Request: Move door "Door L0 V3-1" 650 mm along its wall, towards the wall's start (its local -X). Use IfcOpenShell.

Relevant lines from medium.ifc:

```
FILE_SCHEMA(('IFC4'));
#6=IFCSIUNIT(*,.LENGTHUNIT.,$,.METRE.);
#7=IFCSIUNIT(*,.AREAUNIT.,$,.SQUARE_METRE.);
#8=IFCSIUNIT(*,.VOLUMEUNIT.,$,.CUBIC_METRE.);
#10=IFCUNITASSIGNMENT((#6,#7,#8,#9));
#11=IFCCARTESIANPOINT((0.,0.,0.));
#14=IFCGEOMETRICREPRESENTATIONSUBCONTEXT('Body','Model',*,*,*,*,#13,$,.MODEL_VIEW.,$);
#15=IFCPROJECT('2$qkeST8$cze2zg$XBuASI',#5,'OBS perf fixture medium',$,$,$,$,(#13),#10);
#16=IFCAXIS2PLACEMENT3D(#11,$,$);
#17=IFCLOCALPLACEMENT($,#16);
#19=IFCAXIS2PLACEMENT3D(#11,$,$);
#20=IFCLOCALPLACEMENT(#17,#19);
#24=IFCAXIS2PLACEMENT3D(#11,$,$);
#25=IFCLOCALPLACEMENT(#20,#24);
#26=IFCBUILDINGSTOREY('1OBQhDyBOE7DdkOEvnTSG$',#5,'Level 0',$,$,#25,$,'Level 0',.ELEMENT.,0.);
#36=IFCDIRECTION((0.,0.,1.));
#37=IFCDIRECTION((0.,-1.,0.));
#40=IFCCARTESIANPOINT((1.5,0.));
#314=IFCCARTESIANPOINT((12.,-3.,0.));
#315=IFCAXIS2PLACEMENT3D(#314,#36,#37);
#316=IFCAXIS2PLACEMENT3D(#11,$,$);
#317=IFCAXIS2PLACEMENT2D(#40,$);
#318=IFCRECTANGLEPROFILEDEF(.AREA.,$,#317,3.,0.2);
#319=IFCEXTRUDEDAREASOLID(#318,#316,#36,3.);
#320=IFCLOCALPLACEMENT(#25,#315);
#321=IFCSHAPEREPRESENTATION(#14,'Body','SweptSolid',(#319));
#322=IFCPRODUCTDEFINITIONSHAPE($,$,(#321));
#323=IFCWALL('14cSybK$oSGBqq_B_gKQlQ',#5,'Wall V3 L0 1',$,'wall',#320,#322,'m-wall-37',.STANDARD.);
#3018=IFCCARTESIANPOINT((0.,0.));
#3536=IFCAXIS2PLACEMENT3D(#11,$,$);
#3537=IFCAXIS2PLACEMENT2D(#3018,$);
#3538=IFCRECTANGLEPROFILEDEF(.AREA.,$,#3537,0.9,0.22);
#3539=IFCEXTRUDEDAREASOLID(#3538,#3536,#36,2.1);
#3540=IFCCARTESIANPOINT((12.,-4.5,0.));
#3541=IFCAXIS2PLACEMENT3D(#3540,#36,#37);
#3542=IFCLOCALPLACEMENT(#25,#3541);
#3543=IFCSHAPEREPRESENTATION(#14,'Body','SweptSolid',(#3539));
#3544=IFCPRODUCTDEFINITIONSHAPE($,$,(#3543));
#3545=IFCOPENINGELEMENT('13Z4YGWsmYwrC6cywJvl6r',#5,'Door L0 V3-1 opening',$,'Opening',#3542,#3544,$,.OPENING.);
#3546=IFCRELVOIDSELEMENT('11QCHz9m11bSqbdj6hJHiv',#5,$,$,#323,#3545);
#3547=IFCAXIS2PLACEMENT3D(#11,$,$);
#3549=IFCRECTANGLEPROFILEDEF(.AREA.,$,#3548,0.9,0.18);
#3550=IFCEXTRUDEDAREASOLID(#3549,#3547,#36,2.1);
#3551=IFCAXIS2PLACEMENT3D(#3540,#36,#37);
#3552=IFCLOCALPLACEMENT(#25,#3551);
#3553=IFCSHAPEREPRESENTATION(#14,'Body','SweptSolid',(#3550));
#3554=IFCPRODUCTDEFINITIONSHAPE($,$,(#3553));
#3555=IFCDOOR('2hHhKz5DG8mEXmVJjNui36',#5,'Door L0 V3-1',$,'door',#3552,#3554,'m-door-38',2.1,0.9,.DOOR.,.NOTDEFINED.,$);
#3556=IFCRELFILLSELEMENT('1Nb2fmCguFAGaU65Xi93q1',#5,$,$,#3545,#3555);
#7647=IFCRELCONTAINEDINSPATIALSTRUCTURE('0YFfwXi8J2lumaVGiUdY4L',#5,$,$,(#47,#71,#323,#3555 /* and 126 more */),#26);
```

```python
import ifcopenshell
import ifcopenshell.api.geometry
import ifcopenshell.util.placement

model = ifcopenshell.open("medium.ifc")

door = model.by_guid("2hHhKz5DG8mEXmVJjNui36")
opening = door.FillsVoids[0].RelatingOpeningElement
wall = opening.VoidsElements[0].RelatingBuildingElement

wall_matrix = ifcopenshell.util.placement.get_local_placement(wall.ObjectPlacement)
shift = wall_matrix[:3, 0] * -0.65
before = ifcopenshell.util.placement.get_local_placement(door.ObjectPlacement)[:3, 3].copy()

# The door is not placed relative to its opening, so move both.
for product in (opening, door):
    matrix = ifcopenshell.util.placement.get_local_placement(product.ObjectPlacement)
    matrix[:3, 3] += shift
    ifcopenshell.api.geometry.edit_object_placement(model, product=product, matrix=matrix, is_si=False)

after = ifcopenshell.util.placement.get_local_placement(door.ObjectPlacement)[:3, 3]
print("door moved by", (after - before).round(3) + 0.0)

model.write("medium_v2.ifc")
```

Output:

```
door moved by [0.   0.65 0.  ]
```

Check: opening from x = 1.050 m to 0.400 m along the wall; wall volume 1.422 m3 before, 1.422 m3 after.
